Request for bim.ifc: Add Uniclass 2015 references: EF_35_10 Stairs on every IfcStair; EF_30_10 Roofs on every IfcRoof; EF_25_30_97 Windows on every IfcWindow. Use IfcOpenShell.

First a look at what the model holds.

```python
import ifcopenshell

model = ifcopenshell.open("bim.ifc")
print(model.schema)
print("classifications:", [c.Name for c in model.by_type("IfcClassification")])
for ifc_class in ("IfcDoor", "IfcRoof", "IfcStair", "IfcWall", "IfcWindow"):
    print(ifc_class, len(model.by_type(ifc_class)))
```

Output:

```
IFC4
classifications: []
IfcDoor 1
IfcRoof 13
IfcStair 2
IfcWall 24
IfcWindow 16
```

```python
import ifcopenshell
import ifcopenshell.api.classification

model = ifcopenshell.open("bim.ifc")

system = ifcopenshell.api.classification.add_classification(model, classification="Uniclass 2015")

codes = {
    "IfcStair": ("EF_35_10", "Stairs"),
    "IfcRoof": ("EF_30_10", "Roofs"),
    "IfcWindow": ("EF_25_30_97", "Windows"),
}
for ifc_class, (code, name) in codes.items():
    products = model.by_type(ifc_class)
    ifcopenshell.api.classification.add_reference(
        model, products=products, classification=system, identification=code, name=name
    )
    print(code, len(products))

model.write("bim_rev.ifc")
```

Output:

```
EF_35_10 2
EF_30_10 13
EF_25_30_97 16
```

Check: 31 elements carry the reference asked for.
